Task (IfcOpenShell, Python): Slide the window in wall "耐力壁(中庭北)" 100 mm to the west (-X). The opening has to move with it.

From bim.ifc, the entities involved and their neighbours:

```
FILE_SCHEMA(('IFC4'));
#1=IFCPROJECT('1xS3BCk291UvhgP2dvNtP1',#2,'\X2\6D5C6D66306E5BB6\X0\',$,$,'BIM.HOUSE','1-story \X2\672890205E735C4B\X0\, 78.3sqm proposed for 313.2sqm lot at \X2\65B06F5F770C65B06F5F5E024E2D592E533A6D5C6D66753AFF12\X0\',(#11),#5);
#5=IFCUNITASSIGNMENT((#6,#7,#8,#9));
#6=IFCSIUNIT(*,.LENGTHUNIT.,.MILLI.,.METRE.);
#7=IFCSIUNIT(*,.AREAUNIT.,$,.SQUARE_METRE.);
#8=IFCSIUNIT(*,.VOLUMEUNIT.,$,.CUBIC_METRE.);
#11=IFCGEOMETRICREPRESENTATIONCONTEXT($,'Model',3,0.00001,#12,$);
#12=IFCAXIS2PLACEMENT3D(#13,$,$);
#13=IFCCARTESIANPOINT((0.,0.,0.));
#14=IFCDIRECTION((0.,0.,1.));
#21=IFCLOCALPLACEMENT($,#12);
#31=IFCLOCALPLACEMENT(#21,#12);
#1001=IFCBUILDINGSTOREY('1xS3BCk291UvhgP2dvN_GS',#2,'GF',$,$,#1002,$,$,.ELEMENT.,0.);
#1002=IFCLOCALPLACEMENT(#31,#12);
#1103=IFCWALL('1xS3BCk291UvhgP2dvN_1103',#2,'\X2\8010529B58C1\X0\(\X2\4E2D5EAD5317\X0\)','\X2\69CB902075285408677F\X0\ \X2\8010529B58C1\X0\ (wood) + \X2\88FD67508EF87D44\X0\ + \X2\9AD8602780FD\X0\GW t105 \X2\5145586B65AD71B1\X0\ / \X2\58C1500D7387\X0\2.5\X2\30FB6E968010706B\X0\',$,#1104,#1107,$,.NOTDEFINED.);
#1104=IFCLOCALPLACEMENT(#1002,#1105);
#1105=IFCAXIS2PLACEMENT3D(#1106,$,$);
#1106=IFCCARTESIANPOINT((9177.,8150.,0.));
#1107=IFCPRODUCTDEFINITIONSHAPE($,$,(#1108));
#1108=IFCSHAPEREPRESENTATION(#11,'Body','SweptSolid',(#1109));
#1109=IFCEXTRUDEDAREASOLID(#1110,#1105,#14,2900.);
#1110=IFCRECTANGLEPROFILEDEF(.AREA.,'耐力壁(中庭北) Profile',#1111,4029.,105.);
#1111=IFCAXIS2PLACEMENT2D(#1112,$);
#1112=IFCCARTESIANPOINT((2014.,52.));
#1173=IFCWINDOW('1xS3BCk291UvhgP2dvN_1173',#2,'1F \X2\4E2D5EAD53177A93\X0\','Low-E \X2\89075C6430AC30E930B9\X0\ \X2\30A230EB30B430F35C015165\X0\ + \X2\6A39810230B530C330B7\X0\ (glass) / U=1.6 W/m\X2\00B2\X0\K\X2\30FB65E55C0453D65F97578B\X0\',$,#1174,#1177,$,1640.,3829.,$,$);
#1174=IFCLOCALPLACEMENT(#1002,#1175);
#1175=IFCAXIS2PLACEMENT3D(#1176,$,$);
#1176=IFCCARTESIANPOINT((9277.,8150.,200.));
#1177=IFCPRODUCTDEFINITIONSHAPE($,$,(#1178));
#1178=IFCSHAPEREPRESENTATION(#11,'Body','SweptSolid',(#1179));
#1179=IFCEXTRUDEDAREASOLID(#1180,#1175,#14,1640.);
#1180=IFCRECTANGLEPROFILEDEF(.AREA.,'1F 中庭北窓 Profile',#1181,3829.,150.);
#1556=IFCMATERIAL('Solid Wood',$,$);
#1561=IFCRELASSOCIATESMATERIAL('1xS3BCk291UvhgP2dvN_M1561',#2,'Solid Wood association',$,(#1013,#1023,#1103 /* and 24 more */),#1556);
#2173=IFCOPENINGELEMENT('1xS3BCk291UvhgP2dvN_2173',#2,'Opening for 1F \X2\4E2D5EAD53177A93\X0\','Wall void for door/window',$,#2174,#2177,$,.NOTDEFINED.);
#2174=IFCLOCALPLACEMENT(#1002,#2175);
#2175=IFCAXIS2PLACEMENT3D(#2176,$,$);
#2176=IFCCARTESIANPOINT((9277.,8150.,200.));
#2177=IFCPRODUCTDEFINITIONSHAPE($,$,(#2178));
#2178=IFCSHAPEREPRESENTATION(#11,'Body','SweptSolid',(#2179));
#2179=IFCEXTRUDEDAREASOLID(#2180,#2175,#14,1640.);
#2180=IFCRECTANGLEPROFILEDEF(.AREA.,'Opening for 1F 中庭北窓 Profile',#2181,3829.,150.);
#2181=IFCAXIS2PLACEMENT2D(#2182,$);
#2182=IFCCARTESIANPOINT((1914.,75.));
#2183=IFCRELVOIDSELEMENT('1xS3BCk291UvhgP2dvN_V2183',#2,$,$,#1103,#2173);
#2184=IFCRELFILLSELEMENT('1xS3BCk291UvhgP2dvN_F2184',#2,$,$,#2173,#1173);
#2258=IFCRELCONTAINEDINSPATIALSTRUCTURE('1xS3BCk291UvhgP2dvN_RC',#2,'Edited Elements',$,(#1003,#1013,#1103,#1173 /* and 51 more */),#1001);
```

```python
import ifcopenshell
import ifcopenshell.api.geometry
import ifcopenshell.util.placement
import ifcopenshell.util.unit

model = ifcopenshell.open("bim.ifc")
unit_scale = ifcopenshell.util.unit.calculate_unit_scale(model)

window = model.by_guid("1xS3BCk291UvhgP2dvN_1173")
opening = window.FillsVoids[0].RelatingOpeningElement
wall = opening.VoidsElements[0].RelatingBuildingElement

wall_matrix = ifcopenshell.util.placement.get_local_placement(wall.ObjectPlacement)
shift = wall_matrix[:3, 0] * -0.1 / unit_scale
before = ifcopenshell.util.placement.get_local_placement(window.ObjectPlacement)[:3, 3].copy()

# The window is not placed relative to its opening, so move both.
for product in (opening, window):
    matrix = ifcopenshell.util.placement.get_local_placement(product.ObjectPlacement)
    matrix[:3, 3] += shift
    ifcopenshell.api.geometry.edit_object_placement(model, product=product, matrix=matrix, is_si=False)

after = ifcopenshell.util.placement.get_local_placement(window.ObjectPlacement)[:3, 3]
print("window moved by", (after - before).round(3) + 0.0)

model.write("bim_edited.ifc")
```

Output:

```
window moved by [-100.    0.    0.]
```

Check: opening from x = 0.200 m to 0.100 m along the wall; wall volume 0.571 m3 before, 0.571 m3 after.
